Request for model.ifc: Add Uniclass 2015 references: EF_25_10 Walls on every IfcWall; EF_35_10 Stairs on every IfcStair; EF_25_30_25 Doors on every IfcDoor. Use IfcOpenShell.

First a look at what the model holds.

```python
import ifcopenshell

model = ifcopenshell.open("model.ifc")
print(model.schema)
print("classifications:", [c.Name for c in model.by_type("IfcClassification")])
for ifc_class in ("IfcDoor", "IfcRoof", "IfcStair", "IfcWall", "IfcWindow"):
    print(ifc_class, len(model.by_type(ifc_class)))
```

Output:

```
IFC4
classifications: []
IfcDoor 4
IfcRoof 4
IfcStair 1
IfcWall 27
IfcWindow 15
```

```python
import ifcopenshell
import ifcopenshell.api.classification

model = ifcopenshell.open("model.ifc")

system = ifcopenshell.api.classification.add_classification(model, classification="Uniclass 2015")

codes = {
    "IfcWall": ("EF_25_10", "Walls"),
    "IfcStair": ("EF_35_10", "Stairs"),
    "IfcDoor": ("EF_25_30_25", "Doors"),
}
for ifc_class, (code, name) in codes.items():
    products = model.by_type(ifc_class)
    ifcopenshell.api.classification.add_reference(
        model, products=products, classification=system, identification=code, name=name
    )
    print(code, len(products))

model.write("model-out.ifc")
```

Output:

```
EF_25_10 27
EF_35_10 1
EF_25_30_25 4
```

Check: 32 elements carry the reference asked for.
